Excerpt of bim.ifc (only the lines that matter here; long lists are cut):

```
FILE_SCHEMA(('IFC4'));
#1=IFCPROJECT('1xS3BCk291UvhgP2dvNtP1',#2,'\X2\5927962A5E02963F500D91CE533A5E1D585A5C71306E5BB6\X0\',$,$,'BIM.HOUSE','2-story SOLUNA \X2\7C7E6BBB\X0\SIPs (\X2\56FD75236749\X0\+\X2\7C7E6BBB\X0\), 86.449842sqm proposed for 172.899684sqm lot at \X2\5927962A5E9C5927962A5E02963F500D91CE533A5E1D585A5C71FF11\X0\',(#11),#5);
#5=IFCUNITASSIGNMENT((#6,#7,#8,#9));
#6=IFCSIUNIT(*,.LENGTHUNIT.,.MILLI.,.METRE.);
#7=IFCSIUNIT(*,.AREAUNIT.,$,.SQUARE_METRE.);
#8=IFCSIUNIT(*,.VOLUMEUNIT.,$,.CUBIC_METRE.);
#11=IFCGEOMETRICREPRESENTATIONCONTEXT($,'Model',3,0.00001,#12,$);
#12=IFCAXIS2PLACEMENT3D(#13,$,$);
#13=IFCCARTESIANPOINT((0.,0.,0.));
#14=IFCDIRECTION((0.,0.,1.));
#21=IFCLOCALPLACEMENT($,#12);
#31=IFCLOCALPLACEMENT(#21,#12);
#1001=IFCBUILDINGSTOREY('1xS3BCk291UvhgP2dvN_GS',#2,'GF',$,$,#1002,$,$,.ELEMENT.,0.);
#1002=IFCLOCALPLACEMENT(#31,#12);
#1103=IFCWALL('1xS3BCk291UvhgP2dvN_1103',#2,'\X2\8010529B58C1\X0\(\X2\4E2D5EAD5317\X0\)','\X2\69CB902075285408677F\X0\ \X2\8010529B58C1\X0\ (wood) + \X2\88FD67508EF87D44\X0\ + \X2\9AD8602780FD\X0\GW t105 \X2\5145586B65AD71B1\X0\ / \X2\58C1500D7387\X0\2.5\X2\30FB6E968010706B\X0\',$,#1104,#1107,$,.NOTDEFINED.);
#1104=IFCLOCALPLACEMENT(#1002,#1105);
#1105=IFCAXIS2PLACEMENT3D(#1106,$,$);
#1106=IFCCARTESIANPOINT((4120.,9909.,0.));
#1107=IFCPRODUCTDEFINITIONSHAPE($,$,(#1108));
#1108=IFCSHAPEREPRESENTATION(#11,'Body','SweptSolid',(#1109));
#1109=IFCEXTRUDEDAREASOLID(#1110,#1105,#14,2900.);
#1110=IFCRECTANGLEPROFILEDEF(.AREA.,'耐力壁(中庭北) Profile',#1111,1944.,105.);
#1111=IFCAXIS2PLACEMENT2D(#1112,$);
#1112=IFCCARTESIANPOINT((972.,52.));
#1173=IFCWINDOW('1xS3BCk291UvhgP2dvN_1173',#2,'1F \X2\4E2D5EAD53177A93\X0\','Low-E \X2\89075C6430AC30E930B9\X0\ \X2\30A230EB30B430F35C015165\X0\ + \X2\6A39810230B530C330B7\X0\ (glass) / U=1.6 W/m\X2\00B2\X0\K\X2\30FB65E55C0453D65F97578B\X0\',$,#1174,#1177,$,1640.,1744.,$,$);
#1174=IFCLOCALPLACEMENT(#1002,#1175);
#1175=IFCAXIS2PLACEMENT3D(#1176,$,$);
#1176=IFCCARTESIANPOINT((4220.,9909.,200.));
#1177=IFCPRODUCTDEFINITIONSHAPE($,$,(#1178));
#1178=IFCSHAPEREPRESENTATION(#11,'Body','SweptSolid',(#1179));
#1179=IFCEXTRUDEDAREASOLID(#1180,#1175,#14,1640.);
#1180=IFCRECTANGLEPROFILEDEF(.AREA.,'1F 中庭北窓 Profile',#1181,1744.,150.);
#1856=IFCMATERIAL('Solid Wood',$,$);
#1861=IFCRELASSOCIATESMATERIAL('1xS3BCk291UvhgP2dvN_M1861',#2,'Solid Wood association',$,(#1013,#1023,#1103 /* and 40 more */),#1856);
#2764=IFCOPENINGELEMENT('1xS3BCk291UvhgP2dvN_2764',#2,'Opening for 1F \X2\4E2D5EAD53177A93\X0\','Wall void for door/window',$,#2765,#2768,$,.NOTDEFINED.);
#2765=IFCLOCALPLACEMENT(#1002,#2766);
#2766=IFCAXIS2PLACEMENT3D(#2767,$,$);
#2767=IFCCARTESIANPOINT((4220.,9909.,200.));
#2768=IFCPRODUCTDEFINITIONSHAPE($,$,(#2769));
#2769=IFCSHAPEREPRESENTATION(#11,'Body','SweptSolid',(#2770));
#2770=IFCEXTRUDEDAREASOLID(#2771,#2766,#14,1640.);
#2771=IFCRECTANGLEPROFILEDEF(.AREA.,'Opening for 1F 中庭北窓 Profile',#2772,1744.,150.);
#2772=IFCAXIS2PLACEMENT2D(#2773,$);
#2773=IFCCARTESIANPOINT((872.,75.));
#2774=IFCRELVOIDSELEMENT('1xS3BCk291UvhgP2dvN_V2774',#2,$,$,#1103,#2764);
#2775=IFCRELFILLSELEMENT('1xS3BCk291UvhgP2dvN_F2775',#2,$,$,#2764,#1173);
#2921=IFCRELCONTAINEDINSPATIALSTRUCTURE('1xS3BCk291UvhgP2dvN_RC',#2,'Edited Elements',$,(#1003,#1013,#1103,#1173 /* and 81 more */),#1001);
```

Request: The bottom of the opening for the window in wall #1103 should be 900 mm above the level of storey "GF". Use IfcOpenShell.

```python
import numpy as np
import ifcopenshell
import ifcopenshell.api.geometry
import ifcopenshell.geom
import ifcopenshell.util.element
import ifcopenshell.util.placement
import ifcopenshell.util.shape
import ifcopenshell.util.unit

model = ifcopenshell.open("bim.ifc")
unit_scale = ifcopenshell.util.unit.calculate_unit_scale(model)

window = model.by_guid("1xS3BCk291UvhgP2dvN_1173")
opening = window.FillsVoids[0].RelatingOpeningElement
storey = ifcopenshell.util.element.get_container(window, ifc_class="IfcBuildingStorey")
level = ifcopenshell.util.placement.get_local_placement(storey.ObjectPlacement)[2, 3]

# The opening's origin need not be at the sill, so measure its lowest point.
shape = ifcopenshell.geom.create_shape(ifcopenshell.geom.settings(), opening)
bottom = ifcopenshell.util.shape.get_shape_bottom_elevation(shape, shape.geometry) / unit_scale
dz = level + 900.0 - bottom

shift = np.array([0.0, 0.0, dz])
# The window is not placed relative to its opening, so move both.
for product in (opening, window):
    matrix = ifcopenshell.util.placement.get_local_placement(product.ObjectPlacement)
    matrix[:3, 3] += shift
    ifcopenshell.api.geometry.edit_object_placement(model, product=product, matrix=matrix, is_si=False)

print(f"moved by {dz * unit_scale:+.3f} m")

model.write("bim-out.ifc")
```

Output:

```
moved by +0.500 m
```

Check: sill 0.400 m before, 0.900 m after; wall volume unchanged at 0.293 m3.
